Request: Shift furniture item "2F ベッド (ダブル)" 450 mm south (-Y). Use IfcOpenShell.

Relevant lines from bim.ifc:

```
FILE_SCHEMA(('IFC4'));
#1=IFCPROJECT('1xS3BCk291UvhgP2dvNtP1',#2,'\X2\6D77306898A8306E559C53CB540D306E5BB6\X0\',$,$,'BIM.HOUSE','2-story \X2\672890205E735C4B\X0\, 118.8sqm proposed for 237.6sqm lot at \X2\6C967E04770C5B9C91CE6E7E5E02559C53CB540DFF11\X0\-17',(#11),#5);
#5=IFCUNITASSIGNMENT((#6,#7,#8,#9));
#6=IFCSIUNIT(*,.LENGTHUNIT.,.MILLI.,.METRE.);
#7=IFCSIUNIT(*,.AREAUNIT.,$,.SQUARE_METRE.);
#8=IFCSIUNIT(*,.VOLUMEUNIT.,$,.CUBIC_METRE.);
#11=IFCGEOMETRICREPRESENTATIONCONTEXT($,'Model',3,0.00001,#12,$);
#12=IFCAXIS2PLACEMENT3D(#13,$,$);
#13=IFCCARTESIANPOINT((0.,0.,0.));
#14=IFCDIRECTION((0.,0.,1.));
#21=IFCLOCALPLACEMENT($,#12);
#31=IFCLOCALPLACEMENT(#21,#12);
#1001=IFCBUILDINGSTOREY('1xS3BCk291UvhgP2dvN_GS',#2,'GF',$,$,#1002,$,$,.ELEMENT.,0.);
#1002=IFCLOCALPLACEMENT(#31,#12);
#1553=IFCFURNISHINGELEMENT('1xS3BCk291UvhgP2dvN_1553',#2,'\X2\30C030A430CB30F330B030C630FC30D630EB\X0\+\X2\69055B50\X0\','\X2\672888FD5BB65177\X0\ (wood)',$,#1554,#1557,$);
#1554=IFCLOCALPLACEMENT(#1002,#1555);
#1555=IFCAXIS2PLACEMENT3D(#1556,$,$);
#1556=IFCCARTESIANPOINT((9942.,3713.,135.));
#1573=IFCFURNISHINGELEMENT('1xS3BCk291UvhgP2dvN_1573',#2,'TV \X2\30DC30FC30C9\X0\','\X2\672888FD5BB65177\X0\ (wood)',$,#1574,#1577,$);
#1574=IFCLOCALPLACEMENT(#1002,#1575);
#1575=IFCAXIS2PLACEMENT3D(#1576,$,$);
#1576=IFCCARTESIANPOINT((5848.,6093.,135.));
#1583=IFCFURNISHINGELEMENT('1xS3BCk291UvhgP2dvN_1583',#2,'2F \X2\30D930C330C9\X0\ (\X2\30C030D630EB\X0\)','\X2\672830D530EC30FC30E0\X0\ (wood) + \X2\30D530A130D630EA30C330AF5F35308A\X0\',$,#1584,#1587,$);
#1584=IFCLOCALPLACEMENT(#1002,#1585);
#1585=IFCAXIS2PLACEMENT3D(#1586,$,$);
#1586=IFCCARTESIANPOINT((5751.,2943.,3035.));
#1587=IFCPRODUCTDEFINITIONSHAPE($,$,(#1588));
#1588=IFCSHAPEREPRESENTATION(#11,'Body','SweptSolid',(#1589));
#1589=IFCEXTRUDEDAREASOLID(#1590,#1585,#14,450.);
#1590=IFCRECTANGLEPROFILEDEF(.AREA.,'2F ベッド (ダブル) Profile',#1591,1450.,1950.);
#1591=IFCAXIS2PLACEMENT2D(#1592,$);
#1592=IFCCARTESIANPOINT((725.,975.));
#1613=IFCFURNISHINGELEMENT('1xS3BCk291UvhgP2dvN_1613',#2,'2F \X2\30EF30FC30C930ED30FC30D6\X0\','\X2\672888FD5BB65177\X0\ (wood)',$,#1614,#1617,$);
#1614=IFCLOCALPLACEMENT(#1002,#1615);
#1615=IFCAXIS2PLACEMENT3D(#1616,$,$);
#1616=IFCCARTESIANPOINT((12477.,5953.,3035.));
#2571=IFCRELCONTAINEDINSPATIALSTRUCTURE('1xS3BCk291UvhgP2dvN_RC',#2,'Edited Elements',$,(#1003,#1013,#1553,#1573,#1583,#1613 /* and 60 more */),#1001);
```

```python
import ifcopenshell
import ifcopenshell.api.geometry
import ifcopenshell.util.placement
import ifcopenshell.util.unit

model = ifcopenshell.open("bim.ifc")
unit_scale = ifcopenshell.util.unit.calculate_unit_scale(model)

item = model.by_guid("1xS3BCk291UvhgP2dvN_1583")
matrix = ifcopenshell.util.placement.get_local_placement(item.ObjectPlacement)
matrix[1, 3] -= 0.45 / unit_scale
ifcopenshell.api.geometry.edit_object_placement(model, product=item, matrix=matrix, is_si=False)

print(ifcopenshell.util.placement.get_local_placement(item.ObjectPlacement).round(3) + 0.0)

model.write("bim_updated.ifc")
```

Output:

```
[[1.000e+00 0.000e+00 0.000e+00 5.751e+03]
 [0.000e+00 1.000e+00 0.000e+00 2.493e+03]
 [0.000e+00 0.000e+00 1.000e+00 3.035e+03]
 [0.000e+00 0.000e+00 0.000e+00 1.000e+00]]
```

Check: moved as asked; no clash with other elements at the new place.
